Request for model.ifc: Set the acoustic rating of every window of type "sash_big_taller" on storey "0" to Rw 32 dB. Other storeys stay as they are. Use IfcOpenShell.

First a look at what the model holds.

```python
import ifcopenshell
import ifcopenshell.util.element

model = ifcopenshell.open("model.ifc")
print(model.schema)
storey = next(s for s in model.by_type("IfcBuildingStorey") if s.Name == "0")
windows = [e for e in ifcopenshell.util.element.get_decomposition(storey) if e.is_a("IfcWindow")]
seen = {}
for e in windows:
    element_type = ifcopenshell.util.element.get_type(e)
    key = (element_type.Name if element_type != e and element_type else None, ifcopenshell.util.element.get_pset(e, "Pset_WindowCommon", "AcousticRating"))
    seen[key] = seen.get(key, 0) + 1
for (name, value), count in sorted(seen.items(), key=str):
    print(count, "x", name, "|", value)
```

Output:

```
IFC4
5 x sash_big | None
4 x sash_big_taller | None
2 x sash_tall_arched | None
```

```python
import ifcopenshell
import ifcopenshell.api.pset
import ifcopenshell.util.element

model = ifcopenshell.open("model.ifc")

storey = next(s for s in model.by_type("IfcBuildingStorey") if s.Name == "0")
windows = [e for e in ifcopenshell.util.element.get_decomposition(storey) if e.is_a("IfcWindow")]

count = 0
for e in windows:
    element_type = ifcopenshell.util.element.get_type(e)
    if element_type in (None, e) or element_type.Name != "sash_big_taller":
        continue
    # add_pset returns the element's existing set when there is one.
    pset = ifcopenshell.api.pset.add_pset(model, product=e, name="Pset_WindowCommon")
    ifcopenshell.api.pset.edit_pset(model, pset=pset, properties={"AcousticRating": "Rw 32 dB"})
    count += 1

print(count, "windows updated")

model.write("model-out.ifc")
```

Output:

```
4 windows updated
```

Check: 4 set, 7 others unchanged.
